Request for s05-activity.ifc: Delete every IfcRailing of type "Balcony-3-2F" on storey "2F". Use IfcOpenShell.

First a look at what the model holds.

```python
import ifcopenshell
import ifcopenshell.util.element

model = ifcopenshell.open("s05-activity.ifc")
print(model.schema)
storey = next(s for s in model.by_type("IfcBuildingStorey") if s.Name == "2F")
railings = [e for e in ifcopenshell.util.element.get_decomposition(storey) if e.is_a("IfcRailing")]
seen = {}
for e in railings:
    element_type = ifcopenshell.util.element.get_type(e)
    name = element_type.Name if element_type not in (None, e) else None
    seen[name] = seen.get(name, 0) + 1
for name, count in sorted(seen.items(), key=str):
    print(count, "x", name)
```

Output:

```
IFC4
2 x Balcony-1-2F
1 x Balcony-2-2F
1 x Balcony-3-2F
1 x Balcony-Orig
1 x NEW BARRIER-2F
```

```python
import ifcopenshell
import ifcopenshell.api.root
import ifcopenshell.util.element

model = ifcopenshell.open("s05-activity.ifc")

storey = next(s for s in model.by_type("IfcBuildingStorey") if s.Name == "2F")
railings = [e for e in ifcopenshell.util.element.get_decomposition(storey) if e.is_a("IfcRailing")]
targets = [e for e in railings if (t := ifcopenshell.util.element.get_type(e)) not in (None, e) and t.Name == "Balcony-3-2F"]

for e in targets:
    ifcopenshell.api.root.remove_product(model, product=e)
print(len(targets), "removed")

model.write("s05-activity_v2.ifc")
```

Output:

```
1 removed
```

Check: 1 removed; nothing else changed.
